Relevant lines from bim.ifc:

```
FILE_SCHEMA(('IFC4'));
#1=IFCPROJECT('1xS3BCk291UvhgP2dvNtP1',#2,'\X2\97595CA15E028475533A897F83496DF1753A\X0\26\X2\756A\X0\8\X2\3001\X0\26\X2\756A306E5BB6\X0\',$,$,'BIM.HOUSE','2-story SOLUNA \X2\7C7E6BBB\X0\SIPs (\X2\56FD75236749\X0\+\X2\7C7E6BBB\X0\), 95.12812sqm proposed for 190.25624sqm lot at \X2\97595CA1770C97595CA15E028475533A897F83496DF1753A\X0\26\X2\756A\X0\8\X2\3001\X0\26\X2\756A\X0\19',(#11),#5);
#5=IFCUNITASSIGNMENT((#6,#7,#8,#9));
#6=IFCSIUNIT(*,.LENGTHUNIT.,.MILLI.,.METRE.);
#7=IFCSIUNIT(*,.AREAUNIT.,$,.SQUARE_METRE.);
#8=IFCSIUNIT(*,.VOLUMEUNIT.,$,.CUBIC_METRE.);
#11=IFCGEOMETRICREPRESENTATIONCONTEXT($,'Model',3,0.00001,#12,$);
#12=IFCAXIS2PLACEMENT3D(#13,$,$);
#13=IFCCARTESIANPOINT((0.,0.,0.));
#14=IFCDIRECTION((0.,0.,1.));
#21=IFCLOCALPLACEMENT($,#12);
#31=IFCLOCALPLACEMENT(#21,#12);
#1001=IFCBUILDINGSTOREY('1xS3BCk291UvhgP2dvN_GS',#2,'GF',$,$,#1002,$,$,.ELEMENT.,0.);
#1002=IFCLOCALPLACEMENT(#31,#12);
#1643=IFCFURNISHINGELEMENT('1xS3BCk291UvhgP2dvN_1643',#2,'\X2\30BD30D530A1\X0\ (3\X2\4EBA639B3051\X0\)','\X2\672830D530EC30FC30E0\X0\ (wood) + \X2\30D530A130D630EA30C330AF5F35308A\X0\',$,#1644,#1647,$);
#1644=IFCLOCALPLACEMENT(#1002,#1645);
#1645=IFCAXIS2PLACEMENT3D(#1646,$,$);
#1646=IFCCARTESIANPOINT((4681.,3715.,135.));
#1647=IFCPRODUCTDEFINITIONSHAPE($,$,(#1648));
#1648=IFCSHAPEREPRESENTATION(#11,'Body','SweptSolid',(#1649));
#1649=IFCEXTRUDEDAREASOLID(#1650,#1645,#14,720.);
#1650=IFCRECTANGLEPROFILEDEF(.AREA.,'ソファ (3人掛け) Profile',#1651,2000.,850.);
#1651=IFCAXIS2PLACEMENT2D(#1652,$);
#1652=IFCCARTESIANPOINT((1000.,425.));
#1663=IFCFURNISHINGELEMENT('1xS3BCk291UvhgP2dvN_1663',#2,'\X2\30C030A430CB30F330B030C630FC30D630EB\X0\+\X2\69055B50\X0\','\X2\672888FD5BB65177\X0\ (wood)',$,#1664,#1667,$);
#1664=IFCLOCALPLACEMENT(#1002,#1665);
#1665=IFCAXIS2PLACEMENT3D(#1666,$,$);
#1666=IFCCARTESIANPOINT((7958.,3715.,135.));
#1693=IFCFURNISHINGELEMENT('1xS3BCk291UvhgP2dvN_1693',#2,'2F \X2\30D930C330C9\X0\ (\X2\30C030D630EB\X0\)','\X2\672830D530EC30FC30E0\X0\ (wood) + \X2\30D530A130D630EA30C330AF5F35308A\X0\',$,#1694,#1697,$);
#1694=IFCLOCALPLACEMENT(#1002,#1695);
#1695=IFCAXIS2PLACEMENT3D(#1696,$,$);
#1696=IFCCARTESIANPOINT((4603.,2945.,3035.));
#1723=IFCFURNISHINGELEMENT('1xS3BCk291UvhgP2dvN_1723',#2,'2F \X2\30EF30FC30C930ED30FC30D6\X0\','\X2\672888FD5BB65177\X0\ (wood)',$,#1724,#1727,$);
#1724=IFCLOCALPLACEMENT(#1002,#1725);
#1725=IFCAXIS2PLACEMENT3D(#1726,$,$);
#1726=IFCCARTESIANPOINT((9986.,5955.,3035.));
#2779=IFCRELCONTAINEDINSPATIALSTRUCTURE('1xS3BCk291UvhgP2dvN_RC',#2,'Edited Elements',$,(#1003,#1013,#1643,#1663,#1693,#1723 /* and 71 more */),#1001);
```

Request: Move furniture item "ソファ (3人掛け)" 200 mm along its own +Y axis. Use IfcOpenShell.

```python
import ifcopenshell
import ifcopenshell.api.geometry
import ifcopenshell.util.placement

model = ifcopenshell.open("bim.ifc")

item = model.by_guid("1xS3BCk291UvhgP2dvN_1643")
matrix = ifcopenshell.util.placement.get_local_placement(item.ObjectPlacement)
matrix[:3, 3] += matrix[:3, 1] * 200.0
ifcopenshell.api.geometry.edit_object_placement(model, product=item, matrix=matrix, is_si=False)

print(ifcopenshell.util.placement.get_local_placement(item.ObjectPlacement).round(3) + 0.0)

model.write("bim_v2.ifc")
```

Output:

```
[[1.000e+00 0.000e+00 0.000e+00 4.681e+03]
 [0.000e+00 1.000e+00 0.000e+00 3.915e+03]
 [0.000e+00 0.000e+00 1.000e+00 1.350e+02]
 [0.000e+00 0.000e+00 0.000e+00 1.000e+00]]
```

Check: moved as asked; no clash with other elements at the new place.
